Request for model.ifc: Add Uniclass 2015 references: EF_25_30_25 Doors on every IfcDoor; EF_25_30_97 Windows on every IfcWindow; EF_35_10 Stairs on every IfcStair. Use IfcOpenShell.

First a look at what the model holds.

```python
import ifcopenshell

model = ifcopenshell.open("model.ifc")
print(model.schema)
print("classifications:", [c.Name for c in model.by_type("IfcClassification")])
for ifc_class in ("IfcDoor", "IfcRoof", "IfcStair", "IfcWall", "IfcWindow"):
    print(ifc_class, len(model.by_type(ifc_class)))
```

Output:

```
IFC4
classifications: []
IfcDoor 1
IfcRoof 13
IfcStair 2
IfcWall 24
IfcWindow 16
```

```python
import ifcopenshell
import ifcopenshell.api.classification

model = ifcopenshell.open("model.ifc")

system = ifcopenshell.api.classification.add_classification(model, classification="Uniclass 2015")

codes = {
    "IfcDoor": ("EF_25_30_25", "Doors"),
    "IfcWindow": ("EF_25_30_97", "Windows"),
    "IfcStair": ("EF_35_10", "Stairs"),
}
for ifc_class, (code, name) in codes.items():
    products = model.by_type(ifc_class)
    ifcopenshell.api.classification.add_reference(
        model, products=products, classification=system, identification=code, name=name
    )
    print(code, len(products))

model.write("model_v2.ifc")
```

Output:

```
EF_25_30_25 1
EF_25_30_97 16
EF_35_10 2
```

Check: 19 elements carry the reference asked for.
